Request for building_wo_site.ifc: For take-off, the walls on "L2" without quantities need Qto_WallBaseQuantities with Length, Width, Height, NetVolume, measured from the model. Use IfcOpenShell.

First a look at what the model holds.

```python
import ifcopenshell
import ifcopenshell.util.element
import ifcopenshell.util.unit

model = ifcopenshell.open("building_wo_site.ifc")
print(model.schema)
for unit_type in ("LENGTHUNIT", "AREAUNIT", "VOLUMEUNIT"):
    print(unit_type, ifcopenshell.util.unit.calculate_unit_scale(model, unit_type))
storey = next(s for s in model.by_type("IfcBuildingStorey") if s.Name == "L2")
walls = [e for e in ifcopenshell.util.element.get_decomposition(storey) if e.is_a("IfcWall")]
for e in sorted(walls, key=lambda e: e.id()):
    print(e.id(), e.is_a(), e.Name, list(ifcopenshell.util.element.get_psets(e, qtos_only=True)), sep=" | ")
```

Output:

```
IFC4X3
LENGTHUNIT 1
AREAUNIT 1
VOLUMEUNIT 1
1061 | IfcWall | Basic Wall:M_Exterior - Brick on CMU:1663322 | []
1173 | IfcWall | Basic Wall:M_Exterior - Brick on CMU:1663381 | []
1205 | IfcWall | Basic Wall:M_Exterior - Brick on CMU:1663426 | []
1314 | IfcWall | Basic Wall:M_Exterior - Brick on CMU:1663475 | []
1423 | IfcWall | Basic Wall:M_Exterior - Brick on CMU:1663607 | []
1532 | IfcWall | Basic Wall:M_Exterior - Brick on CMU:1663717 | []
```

```python
import ifcopenshell
import ifcopenshell.api.pset
import ifcopenshell.geom
import ifcopenshell.util.element
import ifcopenshell.util.shape
import ifcopenshell.util.unit

model = ifcopenshell.open("building_wo_site.ifc")
unit_scale = ifcopenshell.util.unit.calculate_unit_scale(model)
volume_scale = ifcopenshell.util.unit.calculate_unit_scale(model, "VOLUMEUNIT")
settings = ifcopenshell.geom.settings()

storey = next(s for s in model.by_type("IfcBuildingStorey") if s.Name == "L2")
walls = [e for e in ifcopenshell.util.element.get_decomposition(storey) if e.is_a("IfcWall")]

for e in sorted(walls, key=lambda e: e.id()):
    if ifcopenshell.util.element.get_psets(e, qtos_only=True, should_inherit=False):
        continue
    # Geometry comes back in metres, in the element's own axes.
    shape = ifcopenshell.geom.create_shape(settings, e)
    values = {
        "Length": ifcopenshell.util.shape.get_x(shape.geometry) / unit_scale,
        "Width": ifcopenshell.util.shape.get_y(shape.geometry) / unit_scale,
        "Height": ifcopenshell.util.shape.get_z(shape.geometry) / unit_scale,
        "NetVolume": ifcopenshell.util.shape.get_volume(shape.geometry) / volume_scale,
    }
    qto = ifcopenshell.api.pset.add_qto(model, product=e, name="Qto_WallBaseQuantities")
    ifcopenshell.api.pset.edit_qto(model, qto=qto, properties=values)
    print(e.id(), {k: round(v, 3) for k, v in values.items()})

model.write("building_wo_site_rev.ifc")
```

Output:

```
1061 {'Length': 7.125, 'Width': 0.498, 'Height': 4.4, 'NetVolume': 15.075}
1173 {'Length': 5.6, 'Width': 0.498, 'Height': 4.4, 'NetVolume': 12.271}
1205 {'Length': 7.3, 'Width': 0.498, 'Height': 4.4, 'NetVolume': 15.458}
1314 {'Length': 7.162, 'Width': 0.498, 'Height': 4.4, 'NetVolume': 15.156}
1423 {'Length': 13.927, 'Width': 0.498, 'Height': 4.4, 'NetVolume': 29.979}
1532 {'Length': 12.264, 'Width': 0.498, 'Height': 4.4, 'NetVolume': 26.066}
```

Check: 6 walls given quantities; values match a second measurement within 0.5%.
